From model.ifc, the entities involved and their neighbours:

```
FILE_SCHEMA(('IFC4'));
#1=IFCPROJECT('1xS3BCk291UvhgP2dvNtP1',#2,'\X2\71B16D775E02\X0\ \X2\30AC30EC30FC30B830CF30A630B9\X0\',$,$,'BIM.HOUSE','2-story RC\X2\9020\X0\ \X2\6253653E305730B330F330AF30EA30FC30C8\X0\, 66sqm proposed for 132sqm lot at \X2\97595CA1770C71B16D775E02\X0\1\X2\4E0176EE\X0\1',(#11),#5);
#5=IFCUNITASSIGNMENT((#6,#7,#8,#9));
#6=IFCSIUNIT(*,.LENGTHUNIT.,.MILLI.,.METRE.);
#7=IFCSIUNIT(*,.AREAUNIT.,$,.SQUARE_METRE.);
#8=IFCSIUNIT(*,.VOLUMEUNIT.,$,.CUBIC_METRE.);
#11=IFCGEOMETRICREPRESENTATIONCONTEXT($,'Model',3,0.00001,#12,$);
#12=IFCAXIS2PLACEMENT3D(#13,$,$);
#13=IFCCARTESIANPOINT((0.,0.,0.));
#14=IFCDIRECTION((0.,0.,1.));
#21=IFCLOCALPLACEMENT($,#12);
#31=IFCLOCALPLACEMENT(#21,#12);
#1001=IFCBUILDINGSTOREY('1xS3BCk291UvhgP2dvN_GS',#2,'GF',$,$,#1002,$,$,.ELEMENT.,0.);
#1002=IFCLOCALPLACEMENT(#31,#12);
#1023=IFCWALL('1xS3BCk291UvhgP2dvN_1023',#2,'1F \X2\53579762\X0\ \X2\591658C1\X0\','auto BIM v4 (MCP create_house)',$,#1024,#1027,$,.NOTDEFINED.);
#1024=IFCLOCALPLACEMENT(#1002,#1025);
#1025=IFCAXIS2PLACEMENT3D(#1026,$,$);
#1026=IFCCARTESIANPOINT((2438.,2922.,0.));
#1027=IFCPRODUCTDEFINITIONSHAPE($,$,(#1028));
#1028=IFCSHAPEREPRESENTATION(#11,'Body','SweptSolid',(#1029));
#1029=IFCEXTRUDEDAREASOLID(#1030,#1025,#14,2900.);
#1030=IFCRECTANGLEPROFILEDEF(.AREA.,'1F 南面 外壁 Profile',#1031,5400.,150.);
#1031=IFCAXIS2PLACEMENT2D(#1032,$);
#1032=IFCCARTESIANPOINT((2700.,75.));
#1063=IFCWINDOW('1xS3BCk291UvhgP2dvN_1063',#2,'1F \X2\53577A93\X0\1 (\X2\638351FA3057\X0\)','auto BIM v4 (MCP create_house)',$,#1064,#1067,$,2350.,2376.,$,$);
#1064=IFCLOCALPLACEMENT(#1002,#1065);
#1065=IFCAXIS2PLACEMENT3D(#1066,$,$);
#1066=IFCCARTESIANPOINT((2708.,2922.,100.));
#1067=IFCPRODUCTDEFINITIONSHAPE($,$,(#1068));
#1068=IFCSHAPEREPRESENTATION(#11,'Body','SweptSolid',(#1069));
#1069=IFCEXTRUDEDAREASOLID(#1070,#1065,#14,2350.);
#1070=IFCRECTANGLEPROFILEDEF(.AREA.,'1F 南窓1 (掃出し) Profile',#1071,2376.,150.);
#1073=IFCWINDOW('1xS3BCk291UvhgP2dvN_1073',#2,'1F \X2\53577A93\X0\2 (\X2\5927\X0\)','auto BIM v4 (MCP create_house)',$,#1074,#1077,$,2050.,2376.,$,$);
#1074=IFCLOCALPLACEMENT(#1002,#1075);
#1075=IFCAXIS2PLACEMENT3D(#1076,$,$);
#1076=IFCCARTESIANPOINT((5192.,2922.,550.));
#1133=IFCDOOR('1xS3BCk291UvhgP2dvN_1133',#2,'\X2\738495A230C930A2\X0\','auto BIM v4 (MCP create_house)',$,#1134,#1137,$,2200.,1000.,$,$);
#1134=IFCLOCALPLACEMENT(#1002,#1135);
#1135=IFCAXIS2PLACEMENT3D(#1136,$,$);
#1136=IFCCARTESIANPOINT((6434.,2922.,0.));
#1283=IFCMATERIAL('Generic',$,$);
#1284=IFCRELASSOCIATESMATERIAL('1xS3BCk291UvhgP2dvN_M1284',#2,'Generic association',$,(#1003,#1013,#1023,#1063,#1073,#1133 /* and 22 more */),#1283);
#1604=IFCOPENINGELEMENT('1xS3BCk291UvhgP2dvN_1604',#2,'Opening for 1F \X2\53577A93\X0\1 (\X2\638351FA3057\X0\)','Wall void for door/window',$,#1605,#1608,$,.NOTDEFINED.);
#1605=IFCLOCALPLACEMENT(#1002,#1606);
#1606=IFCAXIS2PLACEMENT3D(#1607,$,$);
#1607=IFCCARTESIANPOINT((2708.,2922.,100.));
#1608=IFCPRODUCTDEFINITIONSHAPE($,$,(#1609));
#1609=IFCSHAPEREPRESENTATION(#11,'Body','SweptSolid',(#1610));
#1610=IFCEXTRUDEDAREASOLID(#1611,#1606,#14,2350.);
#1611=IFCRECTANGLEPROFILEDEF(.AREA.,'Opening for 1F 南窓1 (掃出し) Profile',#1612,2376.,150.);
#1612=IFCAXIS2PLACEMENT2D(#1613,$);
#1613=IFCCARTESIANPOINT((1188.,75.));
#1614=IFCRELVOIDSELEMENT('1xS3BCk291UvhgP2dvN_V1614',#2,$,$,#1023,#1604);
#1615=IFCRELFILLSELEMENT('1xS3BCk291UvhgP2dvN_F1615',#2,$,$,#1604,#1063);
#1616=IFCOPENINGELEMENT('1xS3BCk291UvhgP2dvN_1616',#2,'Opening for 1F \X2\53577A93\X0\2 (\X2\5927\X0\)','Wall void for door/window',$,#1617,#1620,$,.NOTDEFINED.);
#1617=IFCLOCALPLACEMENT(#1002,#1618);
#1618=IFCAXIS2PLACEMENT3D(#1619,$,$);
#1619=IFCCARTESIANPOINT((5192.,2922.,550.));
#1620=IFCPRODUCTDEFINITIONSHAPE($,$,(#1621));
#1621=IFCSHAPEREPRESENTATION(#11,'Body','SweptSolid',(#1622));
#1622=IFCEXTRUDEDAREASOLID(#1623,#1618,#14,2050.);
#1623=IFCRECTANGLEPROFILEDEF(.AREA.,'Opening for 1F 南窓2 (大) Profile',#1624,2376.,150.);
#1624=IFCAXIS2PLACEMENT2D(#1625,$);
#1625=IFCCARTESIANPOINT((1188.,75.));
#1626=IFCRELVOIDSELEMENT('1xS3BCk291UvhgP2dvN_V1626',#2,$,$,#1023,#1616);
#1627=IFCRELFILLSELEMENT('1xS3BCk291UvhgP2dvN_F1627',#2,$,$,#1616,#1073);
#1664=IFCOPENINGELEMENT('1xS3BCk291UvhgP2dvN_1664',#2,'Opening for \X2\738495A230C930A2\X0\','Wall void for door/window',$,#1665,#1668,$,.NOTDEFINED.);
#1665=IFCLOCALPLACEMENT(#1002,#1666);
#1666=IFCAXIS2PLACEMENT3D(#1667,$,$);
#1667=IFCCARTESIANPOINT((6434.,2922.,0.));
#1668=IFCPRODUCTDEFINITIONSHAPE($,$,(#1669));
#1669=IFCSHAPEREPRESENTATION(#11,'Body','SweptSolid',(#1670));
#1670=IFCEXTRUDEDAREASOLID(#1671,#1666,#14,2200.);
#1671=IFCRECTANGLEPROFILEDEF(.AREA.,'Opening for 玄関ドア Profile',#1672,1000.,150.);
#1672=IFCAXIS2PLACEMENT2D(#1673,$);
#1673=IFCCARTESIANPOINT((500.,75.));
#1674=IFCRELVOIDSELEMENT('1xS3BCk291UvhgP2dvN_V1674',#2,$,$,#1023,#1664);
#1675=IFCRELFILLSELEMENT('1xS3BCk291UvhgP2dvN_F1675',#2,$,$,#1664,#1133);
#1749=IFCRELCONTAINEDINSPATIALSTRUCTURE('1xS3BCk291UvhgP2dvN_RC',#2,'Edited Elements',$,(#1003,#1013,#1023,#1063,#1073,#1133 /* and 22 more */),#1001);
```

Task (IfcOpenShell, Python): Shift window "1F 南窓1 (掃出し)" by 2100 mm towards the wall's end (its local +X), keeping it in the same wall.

```python
import ifcopenshell
import ifcopenshell.api.geometry
import ifcopenshell.util.placement
import ifcopenshell.util.unit

model = ifcopenshell.open("model.ifc")
unit_scale = ifcopenshell.util.unit.calculate_unit_scale(model)

window = model.by_id(1063)
opening = window.FillsVoids[0].RelatingOpeningElement
wall = opening.VoidsElements[0].RelatingBuildingElement

wall_matrix = ifcopenshell.util.placement.get_local_placement(wall.ObjectPlacement)
shift = wall_matrix[:3, 0] * 2.1 / unit_scale
before = ifcopenshell.util.placement.get_local_placement(window.ObjectPlacement)[:3, 3].copy()

# The window is not placed relative to its opening, so move both.
for product in (opening, window):
    matrix = ifcopenshell.util.placement.get_local_placement(product.ObjectPlacement)
    matrix[:3, 3] += shift
    ifcopenshell.api.geometry.edit_object_placement(model, product=product, matrix=matrix, is_si=False)

after = ifcopenshell.util.placement.get_local_placement(window.ObjectPlacement)[:3, 3]
print("window moved by", (after - before).round(3) + 0.0)

model.write("model_edited.ifc")
```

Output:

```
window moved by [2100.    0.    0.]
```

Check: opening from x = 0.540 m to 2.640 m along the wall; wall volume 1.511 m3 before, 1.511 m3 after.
